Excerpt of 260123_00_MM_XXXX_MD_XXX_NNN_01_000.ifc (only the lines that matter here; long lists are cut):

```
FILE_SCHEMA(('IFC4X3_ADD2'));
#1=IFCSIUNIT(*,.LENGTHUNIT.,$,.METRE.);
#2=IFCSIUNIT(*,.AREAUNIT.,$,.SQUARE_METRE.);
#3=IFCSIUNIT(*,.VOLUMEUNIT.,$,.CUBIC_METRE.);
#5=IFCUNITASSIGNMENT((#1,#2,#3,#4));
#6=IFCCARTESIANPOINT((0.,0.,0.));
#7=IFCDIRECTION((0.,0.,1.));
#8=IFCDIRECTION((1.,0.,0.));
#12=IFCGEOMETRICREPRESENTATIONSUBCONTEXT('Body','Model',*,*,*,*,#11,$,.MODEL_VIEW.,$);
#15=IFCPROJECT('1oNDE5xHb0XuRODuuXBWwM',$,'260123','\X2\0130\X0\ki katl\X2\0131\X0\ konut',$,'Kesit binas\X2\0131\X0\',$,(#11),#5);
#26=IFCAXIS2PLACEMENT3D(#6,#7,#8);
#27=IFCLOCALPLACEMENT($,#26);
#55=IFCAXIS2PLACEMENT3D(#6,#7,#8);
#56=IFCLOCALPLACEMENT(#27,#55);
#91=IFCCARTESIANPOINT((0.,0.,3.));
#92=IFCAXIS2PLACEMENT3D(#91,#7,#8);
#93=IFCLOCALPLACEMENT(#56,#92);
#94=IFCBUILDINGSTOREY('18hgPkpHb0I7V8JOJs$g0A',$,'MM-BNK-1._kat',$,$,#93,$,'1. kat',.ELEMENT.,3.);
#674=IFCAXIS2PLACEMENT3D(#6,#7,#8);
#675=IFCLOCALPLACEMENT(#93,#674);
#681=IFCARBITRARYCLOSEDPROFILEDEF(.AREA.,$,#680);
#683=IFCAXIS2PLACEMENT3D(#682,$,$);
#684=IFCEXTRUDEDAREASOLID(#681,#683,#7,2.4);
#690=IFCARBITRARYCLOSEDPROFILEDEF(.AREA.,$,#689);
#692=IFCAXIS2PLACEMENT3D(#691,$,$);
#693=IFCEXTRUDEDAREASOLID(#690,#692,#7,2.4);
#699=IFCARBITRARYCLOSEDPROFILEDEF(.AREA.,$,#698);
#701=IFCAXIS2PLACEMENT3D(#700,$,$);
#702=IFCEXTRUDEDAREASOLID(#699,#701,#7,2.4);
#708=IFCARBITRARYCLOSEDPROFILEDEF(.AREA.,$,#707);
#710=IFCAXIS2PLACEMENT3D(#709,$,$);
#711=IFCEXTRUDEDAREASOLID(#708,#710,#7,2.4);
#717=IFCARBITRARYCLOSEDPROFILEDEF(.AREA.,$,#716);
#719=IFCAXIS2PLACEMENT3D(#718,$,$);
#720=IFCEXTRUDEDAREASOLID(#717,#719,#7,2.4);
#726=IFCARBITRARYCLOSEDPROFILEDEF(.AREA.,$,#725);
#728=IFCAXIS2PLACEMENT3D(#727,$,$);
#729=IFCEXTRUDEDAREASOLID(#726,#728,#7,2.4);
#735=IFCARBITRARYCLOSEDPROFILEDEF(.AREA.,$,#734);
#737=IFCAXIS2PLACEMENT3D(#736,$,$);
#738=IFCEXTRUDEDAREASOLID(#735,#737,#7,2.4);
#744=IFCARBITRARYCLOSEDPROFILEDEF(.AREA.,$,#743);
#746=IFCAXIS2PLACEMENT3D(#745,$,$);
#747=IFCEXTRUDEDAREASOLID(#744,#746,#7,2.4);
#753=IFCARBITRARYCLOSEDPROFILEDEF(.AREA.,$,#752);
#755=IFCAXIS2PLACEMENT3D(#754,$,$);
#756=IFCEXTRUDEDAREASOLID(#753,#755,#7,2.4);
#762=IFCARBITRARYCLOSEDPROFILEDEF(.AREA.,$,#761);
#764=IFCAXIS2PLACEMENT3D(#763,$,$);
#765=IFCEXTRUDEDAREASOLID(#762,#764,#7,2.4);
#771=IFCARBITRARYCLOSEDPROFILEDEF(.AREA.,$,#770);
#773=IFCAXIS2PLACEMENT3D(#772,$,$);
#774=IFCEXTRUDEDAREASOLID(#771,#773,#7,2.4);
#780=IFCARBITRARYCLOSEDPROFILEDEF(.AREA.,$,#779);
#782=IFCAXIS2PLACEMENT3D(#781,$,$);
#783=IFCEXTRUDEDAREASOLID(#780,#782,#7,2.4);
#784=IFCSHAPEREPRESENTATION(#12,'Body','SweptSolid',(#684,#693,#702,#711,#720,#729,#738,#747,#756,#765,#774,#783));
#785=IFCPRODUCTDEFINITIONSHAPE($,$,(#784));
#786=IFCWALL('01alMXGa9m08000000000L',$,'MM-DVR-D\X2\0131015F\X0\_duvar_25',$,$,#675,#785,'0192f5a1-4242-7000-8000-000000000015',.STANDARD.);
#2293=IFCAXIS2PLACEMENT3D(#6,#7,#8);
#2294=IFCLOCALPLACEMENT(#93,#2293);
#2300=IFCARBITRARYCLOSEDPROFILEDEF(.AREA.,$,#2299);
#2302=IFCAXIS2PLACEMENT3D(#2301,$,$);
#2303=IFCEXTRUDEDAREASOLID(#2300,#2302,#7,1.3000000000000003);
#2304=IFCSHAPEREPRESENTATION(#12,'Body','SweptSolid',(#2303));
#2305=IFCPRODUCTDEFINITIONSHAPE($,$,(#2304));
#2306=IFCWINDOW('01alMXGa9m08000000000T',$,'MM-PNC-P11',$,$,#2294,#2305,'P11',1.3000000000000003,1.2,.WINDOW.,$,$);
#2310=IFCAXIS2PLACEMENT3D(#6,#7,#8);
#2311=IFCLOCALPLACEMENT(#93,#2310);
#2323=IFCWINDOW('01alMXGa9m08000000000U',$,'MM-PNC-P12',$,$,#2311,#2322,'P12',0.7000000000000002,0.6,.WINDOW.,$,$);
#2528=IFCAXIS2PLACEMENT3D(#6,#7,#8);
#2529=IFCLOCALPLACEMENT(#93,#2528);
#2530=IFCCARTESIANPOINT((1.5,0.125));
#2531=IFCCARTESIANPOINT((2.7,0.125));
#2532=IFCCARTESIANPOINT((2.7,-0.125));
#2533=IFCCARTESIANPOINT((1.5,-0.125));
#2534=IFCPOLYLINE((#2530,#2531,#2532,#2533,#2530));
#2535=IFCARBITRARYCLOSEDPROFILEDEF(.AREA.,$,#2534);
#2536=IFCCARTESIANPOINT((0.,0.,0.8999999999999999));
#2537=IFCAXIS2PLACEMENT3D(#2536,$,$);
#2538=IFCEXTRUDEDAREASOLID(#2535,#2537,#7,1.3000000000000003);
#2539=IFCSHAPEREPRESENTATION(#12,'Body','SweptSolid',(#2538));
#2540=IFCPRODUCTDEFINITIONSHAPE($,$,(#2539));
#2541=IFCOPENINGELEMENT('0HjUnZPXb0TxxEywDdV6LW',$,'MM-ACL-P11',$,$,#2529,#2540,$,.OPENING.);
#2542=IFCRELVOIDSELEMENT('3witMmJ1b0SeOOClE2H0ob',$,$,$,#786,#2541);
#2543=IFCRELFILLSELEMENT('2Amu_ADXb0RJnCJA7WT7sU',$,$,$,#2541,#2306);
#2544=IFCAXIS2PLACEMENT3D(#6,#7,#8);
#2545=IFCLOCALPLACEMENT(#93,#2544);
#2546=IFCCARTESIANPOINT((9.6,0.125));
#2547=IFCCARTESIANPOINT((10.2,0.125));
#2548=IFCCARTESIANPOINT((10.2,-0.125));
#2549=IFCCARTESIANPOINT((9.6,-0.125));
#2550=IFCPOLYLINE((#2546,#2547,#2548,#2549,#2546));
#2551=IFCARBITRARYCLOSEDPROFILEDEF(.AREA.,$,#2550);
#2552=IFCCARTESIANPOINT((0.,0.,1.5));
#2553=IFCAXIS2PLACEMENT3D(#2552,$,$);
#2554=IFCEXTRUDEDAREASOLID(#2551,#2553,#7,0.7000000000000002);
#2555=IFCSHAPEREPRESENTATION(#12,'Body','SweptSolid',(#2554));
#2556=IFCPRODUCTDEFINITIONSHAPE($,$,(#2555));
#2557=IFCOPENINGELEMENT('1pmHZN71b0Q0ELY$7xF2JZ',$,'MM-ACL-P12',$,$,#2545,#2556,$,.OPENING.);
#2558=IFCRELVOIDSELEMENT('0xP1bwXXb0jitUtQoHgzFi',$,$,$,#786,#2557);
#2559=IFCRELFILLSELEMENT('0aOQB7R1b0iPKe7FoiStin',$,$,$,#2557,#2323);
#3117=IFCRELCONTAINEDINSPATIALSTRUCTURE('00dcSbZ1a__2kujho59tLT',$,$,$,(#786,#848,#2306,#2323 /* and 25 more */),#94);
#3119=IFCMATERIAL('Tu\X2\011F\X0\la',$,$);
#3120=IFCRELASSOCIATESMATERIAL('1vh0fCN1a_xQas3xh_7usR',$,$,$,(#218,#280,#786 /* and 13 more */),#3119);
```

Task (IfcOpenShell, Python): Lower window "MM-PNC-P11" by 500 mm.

```python
import numpy as np
import ifcopenshell
import ifcopenshell.api.geometry
import ifcopenshell.util.placement
import ifcopenshell.util.unit

model = ifcopenshell.open("260123_00_MM_XXXX_MD_XXX_NNN_01_000.ifc")
unit_scale = ifcopenshell.util.unit.calculate_unit_scale(model)

window = model.by_id(2306)
opening = window.FillsVoids[0].RelatingOpeningElement
dz = -0.5 / unit_scale

shift = np.array([0.0, 0.0, dz])
# The window is not placed relative to its opening, so move both.
for product in (opening, window):
    matrix = ifcopenshell.util.placement.get_local_placement(product.ObjectPlacement)
    matrix[:3, 3] += shift
    ifcopenshell.api.geometry.edit_object_placement(model, product=product, matrix=matrix, is_si=False)

print(f"moved by {dz * unit_scale:+.3f} m")

model.write("260123_00_MM_XXXX_MD_XXX_NNN_01_000_updated.ifc")
```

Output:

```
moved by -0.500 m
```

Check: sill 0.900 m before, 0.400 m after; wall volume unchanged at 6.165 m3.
